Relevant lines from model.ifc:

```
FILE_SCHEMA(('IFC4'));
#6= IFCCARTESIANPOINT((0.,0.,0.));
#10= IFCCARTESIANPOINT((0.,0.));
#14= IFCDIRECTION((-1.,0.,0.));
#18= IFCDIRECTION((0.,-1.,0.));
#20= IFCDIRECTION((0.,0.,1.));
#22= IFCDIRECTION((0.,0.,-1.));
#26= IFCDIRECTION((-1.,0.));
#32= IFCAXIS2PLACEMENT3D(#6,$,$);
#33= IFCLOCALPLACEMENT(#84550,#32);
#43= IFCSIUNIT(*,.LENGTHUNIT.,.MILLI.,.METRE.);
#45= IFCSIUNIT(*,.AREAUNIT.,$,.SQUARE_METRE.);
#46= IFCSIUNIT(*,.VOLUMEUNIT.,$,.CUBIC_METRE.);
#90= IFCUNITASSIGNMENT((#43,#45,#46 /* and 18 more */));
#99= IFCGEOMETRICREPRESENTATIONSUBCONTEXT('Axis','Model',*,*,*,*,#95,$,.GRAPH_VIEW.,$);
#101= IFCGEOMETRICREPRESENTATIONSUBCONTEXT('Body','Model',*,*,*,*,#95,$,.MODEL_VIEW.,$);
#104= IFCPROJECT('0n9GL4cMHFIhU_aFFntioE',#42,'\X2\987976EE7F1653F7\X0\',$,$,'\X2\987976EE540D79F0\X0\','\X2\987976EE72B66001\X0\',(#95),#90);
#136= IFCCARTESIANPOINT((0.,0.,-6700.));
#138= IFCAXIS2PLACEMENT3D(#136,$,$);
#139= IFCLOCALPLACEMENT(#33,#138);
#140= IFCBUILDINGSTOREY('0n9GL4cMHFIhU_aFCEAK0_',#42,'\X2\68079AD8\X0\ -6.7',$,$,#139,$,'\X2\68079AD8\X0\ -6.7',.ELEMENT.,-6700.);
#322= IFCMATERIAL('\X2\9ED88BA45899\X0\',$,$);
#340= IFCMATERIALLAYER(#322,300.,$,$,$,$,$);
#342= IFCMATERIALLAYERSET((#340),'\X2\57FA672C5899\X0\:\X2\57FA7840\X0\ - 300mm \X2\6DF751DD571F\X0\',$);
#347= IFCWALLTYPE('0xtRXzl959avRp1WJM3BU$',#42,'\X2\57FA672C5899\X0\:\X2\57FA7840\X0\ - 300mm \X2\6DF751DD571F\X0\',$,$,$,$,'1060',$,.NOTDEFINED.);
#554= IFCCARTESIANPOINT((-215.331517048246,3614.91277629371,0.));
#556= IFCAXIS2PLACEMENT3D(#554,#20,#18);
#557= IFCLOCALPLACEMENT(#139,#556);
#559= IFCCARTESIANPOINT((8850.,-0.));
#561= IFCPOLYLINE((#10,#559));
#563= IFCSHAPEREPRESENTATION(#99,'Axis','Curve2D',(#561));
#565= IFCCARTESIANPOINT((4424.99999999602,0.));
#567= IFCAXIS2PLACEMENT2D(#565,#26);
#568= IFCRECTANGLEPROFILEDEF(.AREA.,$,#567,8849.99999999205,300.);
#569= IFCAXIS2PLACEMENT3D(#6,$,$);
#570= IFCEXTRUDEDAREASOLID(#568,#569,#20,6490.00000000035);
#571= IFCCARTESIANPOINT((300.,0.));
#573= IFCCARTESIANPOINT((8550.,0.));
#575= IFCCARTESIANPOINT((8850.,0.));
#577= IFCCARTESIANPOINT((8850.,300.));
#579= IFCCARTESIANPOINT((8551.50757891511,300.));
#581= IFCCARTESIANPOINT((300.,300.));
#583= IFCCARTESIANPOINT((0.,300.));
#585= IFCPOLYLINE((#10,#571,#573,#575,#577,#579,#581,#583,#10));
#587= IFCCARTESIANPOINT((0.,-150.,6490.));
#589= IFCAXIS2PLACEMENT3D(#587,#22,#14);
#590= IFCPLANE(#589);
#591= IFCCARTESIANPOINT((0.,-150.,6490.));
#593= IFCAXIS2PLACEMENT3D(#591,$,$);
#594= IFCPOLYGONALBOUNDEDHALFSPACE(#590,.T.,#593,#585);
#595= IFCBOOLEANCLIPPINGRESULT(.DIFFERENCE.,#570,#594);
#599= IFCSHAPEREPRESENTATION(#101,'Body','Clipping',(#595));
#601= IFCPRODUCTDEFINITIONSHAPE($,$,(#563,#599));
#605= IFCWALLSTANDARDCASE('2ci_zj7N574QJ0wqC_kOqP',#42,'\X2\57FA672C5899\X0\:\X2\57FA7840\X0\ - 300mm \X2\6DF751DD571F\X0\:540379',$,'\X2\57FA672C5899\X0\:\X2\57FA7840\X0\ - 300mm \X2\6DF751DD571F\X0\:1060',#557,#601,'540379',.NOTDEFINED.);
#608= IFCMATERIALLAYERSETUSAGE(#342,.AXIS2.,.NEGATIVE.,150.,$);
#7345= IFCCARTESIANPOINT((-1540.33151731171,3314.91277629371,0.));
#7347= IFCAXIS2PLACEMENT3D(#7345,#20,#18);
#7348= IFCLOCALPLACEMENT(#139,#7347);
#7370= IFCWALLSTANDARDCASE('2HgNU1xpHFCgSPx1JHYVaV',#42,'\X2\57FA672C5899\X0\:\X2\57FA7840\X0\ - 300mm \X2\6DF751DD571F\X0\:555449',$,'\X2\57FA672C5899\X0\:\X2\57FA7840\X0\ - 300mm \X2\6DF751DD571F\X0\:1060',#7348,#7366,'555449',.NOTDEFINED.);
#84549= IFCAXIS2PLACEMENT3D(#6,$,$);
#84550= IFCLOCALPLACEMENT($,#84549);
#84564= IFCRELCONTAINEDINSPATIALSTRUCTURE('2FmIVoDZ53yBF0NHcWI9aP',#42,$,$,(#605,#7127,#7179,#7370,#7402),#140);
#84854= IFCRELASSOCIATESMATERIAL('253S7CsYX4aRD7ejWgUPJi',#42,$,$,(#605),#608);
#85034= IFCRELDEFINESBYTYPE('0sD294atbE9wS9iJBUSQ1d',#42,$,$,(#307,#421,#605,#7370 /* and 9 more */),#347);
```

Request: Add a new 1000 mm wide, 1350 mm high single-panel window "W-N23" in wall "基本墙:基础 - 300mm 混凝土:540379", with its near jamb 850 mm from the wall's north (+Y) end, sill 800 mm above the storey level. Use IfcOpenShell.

```python
import numpy as np
import ifcopenshell
import ifcopenshell.api.feature
import ifcopenshell.api.geometry
import ifcopenshell.api.root
import ifcopenshell.api.spatial
import ifcopenshell.geom
import ifcopenshell.util.element
import ifcopenshell.util.placement
import ifcopenshell.util.representation
import ifcopenshell.util.shape
import ifcopenshell.util.unit

model = ifcopenshell.open("model.ifc")
unit_scale = ifcopenshell.util.unit.calculate_unit_scale(model)
settings = ifcopenshell.geom.settings()


def volume(element):
    """Net volume in cubic metres, openings subtracted."""
    shape = ifcopenshell.geom.create_shape(settings, element)
    return ifcopenshell.util.shape.get_volume(shape.geometry)


wall = model.by_guid("2ci_zj7N574QJ0wqC_kOqP")
storey = ifcopenshell.util.element.get_container(wall, ifc_class="IfcBuildingStorey")
context = ifcopenshell.util.representation.get_context(model, "Model", "Body", "MODEL_VIEW")
before = volume(wall)

width, height, from_end, sill = 1, 1.35, 0.85, 0.8  # metres

# The wall runs along its own X axis, and the end named is its -X end.
wall_shape = ifcopenshell.geom.create_shape(settings, wall)
x, y, z = ifcopenshell.util.shape.get_vertices(wall_shape.geometry).T
start = x.min() + from_end
face, thickness = float(y.min()), float(y.max() - y.min())
wall_matrix = ifcopenshell.util.placement.get_local_placement(wall.ObjectPlacement)
level = ifcopenshell.util.placement.get_local_placement(storey.ObjectPlacement)[2, 3]


def in_wall(x, y):
    """Placement at x, y metres in the wall's axes, at sill height."""
    matrix = wall_matrix.copy()
    matrix[:, 3] = wall_matrix @ np.array([x / unit_scale, y / unit_scale, 0.0, 1.0])
    matrix[2, 3] = level + sill / unit_scale
    return matrix


# Opening: a box that overshoots both wall faces by 50 mm.
opening = ifcopenshell.api.root.create_entity(model, ifc_class="IfcOpeningElement", predefined_type="OPENING")
box = ifcopenshell.api.geometry.add_wall_representation(
    model, context=context, length=width, height=height, thickness=thickness + 0.1
)
ifcopenshell.api.geometry.assign_representation(model, product=opening, representation=box)
ifcopenshell.api.geometry.edit_object_placement(model, product=opening, matrix=in_wall(start, face - 0.05), is_si=False)
ifcopenshell.api.feature.add_feature(model, feature=opening, element=wall)

window = ifcopenshell.api.root.create_entity(model, ifc_class="IfcWindow", name="W-N23", predefined_type="WINDOW")
window.OverallWidth, window.OverallHeight = width / unit_scale, height / unit_scale
window.PartitioningType = "SINGLE_PANEL"
body = ifcopenshell.api.geometry.add_window_representation(
    model,
    context=context,
    overall_width=window.OverallWidth,
    overall_height=window.OverallHeight,
    partition_type="SINGLE_PANEL",
)
ifcopenshell.api.geometry.assign_representation(model, product=window, representation=body)
ifcopenshell.api.spatial.assign_container(model, products=[window], relating_structure=storey)
ifcopenshell.api.feature.add_filling(model, opening=opening, element=window)

# Centre the window in the wall's thickness.
ifcopenshell.api.geometry.edit_object_placement(model, product=window, matrix=in_wall(start, face), is_si=False)
window_shape = ifcopenshell.geom.create_shape(settings, window)
depth = ifcopenshell.util.shape.get_vertices(window_shape.geometry)[:, 1]
offset = face + thickness / 2 - (depth.min() + depth.max()) / 2
ifcopenshell.api.geometry.edit_object_placement(model, product=window, matrix=in_wall(start, offset), is_si=False)

after = volume(wall)

print(f"wall volume {before:.3f} -> {after:.3f} m3")

model.write("model_v2.ifc")
```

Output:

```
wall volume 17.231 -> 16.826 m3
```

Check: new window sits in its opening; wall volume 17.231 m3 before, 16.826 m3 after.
